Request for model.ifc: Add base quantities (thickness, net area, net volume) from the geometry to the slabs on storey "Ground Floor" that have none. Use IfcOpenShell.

First a look at what the model holds.

```python
import ifcopenshell
import ifcopenshell.util.element
import ifcopenshell.util.unit

model = ifcopenshell.open("model.ifc")
print(model.schema)
for unit_type in ("LENGTHUNIT", "AREAUNIT", "VOLUMEUNIT"):
    print(unit_type, ifcopenshell.util.unit.calculate_unit_scale(model, unit_type))
storey = next(s for s in model.by_type("IfcBuildingStorey") if s.Name == "Ground Floor")
slabs = [e for e in ifcopenshell.util.element.get_decomposition(storey) if e.is_a("IfcSlab")]
for e in sorted(slabs, key=lambda e: e.id()):
    print(e.id(), e.is_a(), e.Name, list(ifcopenshell.util.element.get_psets(e, qtos_only=True)), sep=" | ")
```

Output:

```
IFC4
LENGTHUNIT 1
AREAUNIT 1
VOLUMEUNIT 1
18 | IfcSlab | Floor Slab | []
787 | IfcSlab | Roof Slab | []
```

```python
import ifcopenshell
import ifcopenshell.api.pset
import ifcopenshell.geom
import ifcopenshell.util.element
import ifcopenshell.util.shape
import ifcopenshell.util.unit

model = ifcopenshell.open("model.ifc")
unit_scale = ifcopenshell.util.unit.calculate_unit_scale(model)
area_scale = ifcopenshell.util.unit.calculate_unit_scale(model, "AREAUNIT")
volume_scale = ifcopenshell.util.unit.calculate_unit_scale(model, "VOLUMEUNIT")
settings = ifcopenshell.geom.settings()

storey = next(s for s in model.by_type("IfcBuildingStorey") if s.Name == "Ground Floor")
slabs = [e for e in ifcopenshell.util.element.get_decomposition(storey) if e.is_a("IfcSlab")]

for e in sorted(slabs, key=lambda e: e.id()):
    if ifcopenshell.util.element.get_psets(e, qtos_only=True, should_inherit=False):
        continue
    # Geometry comes back in metres, in the element's own axes.
    shape = ifcopenshell.geom.create_shape(settings, e)
    values = {
        "Width": ifcopenshell.util.shape.get_z(shape.geometry) / unit_scale,
        "NetArea": ifcopenshell.util.shape.get_footprint_area(shape.geometry) / area_scale,
        "NetVolume": ifcopenshell.util.shape.get_volume(shape.geometry) / volume_scale,
    }
    qto = ifcopenshell.api.pset.add_qto(model, product=e, name="Qto_SlabBaseQuantities")
    ifcopenshell.api.pset.edit_qto(model, qto=qto, properties=values)
    print(e.id(), {k: round(v, 3) for k, v in values.items()})

model.write("model_rev.ifc")
```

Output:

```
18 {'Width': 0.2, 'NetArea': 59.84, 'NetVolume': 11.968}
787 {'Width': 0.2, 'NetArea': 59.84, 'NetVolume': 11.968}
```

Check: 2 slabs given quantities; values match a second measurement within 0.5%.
